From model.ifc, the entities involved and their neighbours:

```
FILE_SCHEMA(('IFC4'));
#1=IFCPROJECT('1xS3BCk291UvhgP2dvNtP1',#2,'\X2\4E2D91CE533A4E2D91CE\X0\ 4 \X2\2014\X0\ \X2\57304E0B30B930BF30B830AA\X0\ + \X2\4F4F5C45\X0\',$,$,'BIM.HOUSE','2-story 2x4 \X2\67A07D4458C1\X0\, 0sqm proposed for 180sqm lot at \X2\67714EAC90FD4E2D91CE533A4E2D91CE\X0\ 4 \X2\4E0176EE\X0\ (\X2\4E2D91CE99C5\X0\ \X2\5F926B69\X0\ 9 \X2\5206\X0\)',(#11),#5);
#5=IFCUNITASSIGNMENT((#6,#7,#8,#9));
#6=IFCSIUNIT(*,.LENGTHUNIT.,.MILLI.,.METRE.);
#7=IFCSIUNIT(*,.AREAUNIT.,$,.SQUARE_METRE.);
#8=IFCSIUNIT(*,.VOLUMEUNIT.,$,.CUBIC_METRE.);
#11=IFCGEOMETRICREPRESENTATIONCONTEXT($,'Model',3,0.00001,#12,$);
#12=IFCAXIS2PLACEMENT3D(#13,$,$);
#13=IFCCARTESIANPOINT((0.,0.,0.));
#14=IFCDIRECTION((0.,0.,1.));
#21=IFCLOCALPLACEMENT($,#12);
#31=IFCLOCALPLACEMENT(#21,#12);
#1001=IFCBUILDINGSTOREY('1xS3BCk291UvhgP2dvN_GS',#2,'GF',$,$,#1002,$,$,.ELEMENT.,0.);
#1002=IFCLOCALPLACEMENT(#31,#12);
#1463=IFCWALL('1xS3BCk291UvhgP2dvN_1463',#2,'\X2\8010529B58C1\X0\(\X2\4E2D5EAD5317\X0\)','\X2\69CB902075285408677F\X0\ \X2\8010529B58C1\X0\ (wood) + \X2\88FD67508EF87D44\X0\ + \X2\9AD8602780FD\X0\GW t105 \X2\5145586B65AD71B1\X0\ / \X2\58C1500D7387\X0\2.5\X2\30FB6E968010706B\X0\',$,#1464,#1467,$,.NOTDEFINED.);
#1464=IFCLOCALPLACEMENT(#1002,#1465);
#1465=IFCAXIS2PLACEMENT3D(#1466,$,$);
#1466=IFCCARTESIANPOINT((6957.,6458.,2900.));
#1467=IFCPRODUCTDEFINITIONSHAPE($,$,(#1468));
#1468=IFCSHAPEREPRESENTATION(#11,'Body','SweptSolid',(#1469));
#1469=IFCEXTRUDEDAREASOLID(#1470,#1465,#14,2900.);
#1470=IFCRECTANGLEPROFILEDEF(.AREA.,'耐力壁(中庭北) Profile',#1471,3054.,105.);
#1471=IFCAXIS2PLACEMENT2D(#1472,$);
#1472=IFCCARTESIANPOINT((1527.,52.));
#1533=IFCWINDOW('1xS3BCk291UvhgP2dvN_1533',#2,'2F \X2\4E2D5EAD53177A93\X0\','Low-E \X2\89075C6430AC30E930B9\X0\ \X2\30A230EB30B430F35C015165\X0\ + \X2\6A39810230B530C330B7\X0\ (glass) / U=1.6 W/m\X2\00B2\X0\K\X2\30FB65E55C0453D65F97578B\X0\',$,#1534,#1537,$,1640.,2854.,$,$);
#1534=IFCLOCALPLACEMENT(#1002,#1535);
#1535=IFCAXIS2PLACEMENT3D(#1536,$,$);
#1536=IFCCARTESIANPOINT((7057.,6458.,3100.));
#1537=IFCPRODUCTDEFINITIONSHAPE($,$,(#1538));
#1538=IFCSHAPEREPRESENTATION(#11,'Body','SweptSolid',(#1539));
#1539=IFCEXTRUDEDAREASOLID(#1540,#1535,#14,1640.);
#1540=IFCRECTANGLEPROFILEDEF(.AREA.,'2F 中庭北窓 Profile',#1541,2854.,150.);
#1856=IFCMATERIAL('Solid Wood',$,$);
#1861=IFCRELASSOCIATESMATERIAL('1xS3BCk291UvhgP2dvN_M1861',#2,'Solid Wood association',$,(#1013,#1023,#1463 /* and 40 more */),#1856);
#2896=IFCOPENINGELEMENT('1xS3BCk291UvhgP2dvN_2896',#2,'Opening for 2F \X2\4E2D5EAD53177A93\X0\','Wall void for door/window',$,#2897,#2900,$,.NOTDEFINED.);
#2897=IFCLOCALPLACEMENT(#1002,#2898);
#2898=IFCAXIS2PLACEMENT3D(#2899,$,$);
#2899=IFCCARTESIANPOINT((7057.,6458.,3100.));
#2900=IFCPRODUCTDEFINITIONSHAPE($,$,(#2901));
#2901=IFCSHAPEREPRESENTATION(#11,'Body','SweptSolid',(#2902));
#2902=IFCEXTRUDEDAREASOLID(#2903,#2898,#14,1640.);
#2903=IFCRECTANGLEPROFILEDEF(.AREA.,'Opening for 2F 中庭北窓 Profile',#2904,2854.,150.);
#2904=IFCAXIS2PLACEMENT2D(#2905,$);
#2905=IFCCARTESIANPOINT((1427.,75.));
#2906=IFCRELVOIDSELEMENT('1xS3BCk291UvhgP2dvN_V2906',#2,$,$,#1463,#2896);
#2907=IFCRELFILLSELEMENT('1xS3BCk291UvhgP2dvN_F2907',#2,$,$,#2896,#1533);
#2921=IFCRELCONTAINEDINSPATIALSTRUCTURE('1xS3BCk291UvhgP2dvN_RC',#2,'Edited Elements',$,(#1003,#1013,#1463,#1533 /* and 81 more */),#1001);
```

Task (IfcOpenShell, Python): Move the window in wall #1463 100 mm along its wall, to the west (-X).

```python
import ifcopenshell
import ifcopenshell.api.geometry
import ifcopenshell.util.placement
import ifcopenshell.util.unit

model = ifcopenshell.open("model.ifc")
unit_scale = ifcopenshell.util.unit.calculate_unit_scale(model)

window = model.by_guid("1xS3BCk291UvhgP2dvN_1533")
opening = window.FillsVoids[0].RelatingOpeningElement
wall = opening.VoidsElements[0].RelatingBuildingElement

wall_matrix = ifcopenshell.util.placement.get_local_placement(wall.ObjectPlacement)
shift = wall_matrix[:3, 0] * -0.1 / unit_scale
before = ifcopenshell.util.placement.get_local_placement(window.ObjectPlacement)[:3, 3].copy()

# The window is not placed relative to its opening, so move both.
for product in (opening, window):
    matrix = ifcopenshell.util.placement.get_local_placement(product.ObjectPlacement)
    matrix[:3, 3] += shift
    ifcopenshell.api.geometry.edit_object_placement(model, product=product, matrix=matrix, is_si=False)

after = ifcopenshell.util.placement.get_local_placement(window.ObjectPlacement)[:3, 3]
print("window moved by", (after - before).round(3) + 0.0)

model.write("model_rev.ifc")
```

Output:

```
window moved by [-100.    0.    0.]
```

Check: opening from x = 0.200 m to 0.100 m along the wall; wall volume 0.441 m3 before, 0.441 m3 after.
